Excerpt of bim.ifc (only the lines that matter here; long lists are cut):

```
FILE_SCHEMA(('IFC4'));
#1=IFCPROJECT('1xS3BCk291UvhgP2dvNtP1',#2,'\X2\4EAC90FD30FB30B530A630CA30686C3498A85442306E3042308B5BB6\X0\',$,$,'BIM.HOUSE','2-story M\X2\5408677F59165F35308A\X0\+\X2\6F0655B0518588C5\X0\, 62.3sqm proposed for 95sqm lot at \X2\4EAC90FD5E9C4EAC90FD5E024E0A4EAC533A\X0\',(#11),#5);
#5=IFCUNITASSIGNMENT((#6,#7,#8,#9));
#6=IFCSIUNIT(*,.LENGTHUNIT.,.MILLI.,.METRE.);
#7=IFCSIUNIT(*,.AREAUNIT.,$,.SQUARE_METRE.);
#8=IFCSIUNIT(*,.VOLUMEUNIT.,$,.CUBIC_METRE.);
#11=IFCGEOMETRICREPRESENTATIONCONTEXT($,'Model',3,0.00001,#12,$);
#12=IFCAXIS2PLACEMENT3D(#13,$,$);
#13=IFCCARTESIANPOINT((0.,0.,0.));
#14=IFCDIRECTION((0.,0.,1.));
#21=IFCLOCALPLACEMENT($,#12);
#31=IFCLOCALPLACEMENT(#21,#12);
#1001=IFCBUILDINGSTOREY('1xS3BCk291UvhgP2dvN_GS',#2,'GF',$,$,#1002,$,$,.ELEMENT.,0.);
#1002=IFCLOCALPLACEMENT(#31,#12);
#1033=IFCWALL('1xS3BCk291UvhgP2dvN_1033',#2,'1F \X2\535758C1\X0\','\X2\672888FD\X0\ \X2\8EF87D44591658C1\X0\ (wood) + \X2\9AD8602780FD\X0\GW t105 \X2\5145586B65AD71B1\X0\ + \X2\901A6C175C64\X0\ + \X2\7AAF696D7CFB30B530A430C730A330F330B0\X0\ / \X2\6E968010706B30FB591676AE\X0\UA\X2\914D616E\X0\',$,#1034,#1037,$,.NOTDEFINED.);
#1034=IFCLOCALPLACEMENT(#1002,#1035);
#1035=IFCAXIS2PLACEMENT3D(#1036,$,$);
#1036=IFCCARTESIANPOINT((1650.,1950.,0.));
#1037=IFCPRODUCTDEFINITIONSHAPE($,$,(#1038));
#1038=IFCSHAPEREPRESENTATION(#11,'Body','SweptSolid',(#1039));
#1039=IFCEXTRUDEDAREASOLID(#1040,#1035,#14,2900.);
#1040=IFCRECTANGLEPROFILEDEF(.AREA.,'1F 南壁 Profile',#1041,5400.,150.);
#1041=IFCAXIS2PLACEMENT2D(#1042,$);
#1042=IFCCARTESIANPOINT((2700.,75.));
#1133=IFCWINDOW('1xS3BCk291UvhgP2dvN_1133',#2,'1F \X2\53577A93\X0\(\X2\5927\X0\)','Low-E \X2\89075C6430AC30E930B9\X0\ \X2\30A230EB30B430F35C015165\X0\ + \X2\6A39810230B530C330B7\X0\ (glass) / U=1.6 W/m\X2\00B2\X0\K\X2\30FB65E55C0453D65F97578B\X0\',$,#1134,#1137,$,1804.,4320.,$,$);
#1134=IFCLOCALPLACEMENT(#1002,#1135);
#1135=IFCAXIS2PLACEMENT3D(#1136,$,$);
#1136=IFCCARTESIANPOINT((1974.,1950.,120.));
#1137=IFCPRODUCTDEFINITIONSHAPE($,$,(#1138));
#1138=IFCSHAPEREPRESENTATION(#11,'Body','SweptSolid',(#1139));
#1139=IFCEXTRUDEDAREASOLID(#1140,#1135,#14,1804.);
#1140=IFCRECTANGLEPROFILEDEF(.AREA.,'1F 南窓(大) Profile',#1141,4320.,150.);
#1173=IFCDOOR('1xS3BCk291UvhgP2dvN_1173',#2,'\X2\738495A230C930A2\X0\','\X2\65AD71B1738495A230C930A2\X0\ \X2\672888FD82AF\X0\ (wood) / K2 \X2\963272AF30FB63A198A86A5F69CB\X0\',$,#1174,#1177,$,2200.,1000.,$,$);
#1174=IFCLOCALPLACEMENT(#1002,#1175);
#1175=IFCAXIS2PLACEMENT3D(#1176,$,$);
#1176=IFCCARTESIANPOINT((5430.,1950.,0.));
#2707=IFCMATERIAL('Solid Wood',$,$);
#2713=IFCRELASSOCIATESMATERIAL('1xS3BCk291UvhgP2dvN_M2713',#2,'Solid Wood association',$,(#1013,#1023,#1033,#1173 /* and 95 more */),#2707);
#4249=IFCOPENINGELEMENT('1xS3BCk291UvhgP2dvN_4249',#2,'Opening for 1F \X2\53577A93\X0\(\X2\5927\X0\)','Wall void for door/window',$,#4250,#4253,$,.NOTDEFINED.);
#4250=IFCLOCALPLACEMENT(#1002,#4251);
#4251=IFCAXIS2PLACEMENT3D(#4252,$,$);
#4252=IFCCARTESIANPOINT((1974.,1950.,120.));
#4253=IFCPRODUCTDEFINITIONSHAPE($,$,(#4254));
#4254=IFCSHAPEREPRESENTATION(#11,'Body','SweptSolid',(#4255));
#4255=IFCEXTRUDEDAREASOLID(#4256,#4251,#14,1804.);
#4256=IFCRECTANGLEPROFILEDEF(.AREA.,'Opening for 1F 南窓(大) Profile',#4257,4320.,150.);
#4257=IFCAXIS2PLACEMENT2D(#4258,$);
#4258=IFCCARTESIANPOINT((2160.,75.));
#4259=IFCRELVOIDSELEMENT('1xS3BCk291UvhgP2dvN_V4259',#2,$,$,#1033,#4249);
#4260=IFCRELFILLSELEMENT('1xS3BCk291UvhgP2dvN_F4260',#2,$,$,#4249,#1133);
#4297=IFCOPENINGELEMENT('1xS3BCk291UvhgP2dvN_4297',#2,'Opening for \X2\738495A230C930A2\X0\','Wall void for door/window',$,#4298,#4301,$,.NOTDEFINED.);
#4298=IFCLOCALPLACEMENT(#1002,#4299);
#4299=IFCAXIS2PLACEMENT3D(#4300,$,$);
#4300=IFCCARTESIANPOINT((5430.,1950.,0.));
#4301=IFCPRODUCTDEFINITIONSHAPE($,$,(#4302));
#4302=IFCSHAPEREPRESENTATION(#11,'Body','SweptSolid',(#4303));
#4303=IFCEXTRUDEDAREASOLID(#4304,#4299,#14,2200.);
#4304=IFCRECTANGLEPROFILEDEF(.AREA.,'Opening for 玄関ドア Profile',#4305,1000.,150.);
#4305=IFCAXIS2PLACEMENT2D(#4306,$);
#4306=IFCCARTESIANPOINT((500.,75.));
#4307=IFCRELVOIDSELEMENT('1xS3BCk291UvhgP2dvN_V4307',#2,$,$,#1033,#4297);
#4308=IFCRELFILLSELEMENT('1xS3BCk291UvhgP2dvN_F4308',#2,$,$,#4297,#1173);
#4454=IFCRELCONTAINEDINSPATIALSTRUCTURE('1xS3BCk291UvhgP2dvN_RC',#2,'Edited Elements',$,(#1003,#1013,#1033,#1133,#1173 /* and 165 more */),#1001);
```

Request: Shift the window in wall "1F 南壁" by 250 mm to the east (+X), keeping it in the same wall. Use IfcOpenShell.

```python
import ifcopenshell
import ifcopenshell.api.geometry
import ifcopenshell.util.placement
import ifcopenshell.util.unit

model = ifcopenshell.open("bim.ifc")
unit_scale = ifcopenshell.util.unit.calculate_unit_scale(model)

window = model.by_guid("1xS3BCk291UvhgP2dvN_1133")
opening = window.FillsVoids[0].RelatingOpeningElement
wall = opening.VoidsElements[0].RelatingBuildingElement

wall_matrix = ifcopenshell.util.placement.get_local_placement(wall.ObjectPlacement)
shift = wall_matrix[:3, 0] * 0.25 / unit_scale
before = ifcopenshell.util.placement.get_local_placement(window.ObjectPlacement)[:3, 3].copy()

# The window is not placed relative to its opening, so move both.
for product in (opening, window):
    matrix = ifcopenshell.util.placement.get_local_placement(product.ObjectPlacement)
    matrix[:3, 3] += shift
    ifcopenshell.api.geometry.edit_object_placement(model, product=product, matrix=matrix, is_si=False)

after = ifcopenshell.util.placement.get_local_placement(window.ObjectPlacement)[:3, 3]
print("window moved by", (after - before).round(3) + 0.0)

model.write("bim-out.ifc")
```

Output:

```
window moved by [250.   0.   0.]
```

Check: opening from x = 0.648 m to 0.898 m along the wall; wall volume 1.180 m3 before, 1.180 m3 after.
